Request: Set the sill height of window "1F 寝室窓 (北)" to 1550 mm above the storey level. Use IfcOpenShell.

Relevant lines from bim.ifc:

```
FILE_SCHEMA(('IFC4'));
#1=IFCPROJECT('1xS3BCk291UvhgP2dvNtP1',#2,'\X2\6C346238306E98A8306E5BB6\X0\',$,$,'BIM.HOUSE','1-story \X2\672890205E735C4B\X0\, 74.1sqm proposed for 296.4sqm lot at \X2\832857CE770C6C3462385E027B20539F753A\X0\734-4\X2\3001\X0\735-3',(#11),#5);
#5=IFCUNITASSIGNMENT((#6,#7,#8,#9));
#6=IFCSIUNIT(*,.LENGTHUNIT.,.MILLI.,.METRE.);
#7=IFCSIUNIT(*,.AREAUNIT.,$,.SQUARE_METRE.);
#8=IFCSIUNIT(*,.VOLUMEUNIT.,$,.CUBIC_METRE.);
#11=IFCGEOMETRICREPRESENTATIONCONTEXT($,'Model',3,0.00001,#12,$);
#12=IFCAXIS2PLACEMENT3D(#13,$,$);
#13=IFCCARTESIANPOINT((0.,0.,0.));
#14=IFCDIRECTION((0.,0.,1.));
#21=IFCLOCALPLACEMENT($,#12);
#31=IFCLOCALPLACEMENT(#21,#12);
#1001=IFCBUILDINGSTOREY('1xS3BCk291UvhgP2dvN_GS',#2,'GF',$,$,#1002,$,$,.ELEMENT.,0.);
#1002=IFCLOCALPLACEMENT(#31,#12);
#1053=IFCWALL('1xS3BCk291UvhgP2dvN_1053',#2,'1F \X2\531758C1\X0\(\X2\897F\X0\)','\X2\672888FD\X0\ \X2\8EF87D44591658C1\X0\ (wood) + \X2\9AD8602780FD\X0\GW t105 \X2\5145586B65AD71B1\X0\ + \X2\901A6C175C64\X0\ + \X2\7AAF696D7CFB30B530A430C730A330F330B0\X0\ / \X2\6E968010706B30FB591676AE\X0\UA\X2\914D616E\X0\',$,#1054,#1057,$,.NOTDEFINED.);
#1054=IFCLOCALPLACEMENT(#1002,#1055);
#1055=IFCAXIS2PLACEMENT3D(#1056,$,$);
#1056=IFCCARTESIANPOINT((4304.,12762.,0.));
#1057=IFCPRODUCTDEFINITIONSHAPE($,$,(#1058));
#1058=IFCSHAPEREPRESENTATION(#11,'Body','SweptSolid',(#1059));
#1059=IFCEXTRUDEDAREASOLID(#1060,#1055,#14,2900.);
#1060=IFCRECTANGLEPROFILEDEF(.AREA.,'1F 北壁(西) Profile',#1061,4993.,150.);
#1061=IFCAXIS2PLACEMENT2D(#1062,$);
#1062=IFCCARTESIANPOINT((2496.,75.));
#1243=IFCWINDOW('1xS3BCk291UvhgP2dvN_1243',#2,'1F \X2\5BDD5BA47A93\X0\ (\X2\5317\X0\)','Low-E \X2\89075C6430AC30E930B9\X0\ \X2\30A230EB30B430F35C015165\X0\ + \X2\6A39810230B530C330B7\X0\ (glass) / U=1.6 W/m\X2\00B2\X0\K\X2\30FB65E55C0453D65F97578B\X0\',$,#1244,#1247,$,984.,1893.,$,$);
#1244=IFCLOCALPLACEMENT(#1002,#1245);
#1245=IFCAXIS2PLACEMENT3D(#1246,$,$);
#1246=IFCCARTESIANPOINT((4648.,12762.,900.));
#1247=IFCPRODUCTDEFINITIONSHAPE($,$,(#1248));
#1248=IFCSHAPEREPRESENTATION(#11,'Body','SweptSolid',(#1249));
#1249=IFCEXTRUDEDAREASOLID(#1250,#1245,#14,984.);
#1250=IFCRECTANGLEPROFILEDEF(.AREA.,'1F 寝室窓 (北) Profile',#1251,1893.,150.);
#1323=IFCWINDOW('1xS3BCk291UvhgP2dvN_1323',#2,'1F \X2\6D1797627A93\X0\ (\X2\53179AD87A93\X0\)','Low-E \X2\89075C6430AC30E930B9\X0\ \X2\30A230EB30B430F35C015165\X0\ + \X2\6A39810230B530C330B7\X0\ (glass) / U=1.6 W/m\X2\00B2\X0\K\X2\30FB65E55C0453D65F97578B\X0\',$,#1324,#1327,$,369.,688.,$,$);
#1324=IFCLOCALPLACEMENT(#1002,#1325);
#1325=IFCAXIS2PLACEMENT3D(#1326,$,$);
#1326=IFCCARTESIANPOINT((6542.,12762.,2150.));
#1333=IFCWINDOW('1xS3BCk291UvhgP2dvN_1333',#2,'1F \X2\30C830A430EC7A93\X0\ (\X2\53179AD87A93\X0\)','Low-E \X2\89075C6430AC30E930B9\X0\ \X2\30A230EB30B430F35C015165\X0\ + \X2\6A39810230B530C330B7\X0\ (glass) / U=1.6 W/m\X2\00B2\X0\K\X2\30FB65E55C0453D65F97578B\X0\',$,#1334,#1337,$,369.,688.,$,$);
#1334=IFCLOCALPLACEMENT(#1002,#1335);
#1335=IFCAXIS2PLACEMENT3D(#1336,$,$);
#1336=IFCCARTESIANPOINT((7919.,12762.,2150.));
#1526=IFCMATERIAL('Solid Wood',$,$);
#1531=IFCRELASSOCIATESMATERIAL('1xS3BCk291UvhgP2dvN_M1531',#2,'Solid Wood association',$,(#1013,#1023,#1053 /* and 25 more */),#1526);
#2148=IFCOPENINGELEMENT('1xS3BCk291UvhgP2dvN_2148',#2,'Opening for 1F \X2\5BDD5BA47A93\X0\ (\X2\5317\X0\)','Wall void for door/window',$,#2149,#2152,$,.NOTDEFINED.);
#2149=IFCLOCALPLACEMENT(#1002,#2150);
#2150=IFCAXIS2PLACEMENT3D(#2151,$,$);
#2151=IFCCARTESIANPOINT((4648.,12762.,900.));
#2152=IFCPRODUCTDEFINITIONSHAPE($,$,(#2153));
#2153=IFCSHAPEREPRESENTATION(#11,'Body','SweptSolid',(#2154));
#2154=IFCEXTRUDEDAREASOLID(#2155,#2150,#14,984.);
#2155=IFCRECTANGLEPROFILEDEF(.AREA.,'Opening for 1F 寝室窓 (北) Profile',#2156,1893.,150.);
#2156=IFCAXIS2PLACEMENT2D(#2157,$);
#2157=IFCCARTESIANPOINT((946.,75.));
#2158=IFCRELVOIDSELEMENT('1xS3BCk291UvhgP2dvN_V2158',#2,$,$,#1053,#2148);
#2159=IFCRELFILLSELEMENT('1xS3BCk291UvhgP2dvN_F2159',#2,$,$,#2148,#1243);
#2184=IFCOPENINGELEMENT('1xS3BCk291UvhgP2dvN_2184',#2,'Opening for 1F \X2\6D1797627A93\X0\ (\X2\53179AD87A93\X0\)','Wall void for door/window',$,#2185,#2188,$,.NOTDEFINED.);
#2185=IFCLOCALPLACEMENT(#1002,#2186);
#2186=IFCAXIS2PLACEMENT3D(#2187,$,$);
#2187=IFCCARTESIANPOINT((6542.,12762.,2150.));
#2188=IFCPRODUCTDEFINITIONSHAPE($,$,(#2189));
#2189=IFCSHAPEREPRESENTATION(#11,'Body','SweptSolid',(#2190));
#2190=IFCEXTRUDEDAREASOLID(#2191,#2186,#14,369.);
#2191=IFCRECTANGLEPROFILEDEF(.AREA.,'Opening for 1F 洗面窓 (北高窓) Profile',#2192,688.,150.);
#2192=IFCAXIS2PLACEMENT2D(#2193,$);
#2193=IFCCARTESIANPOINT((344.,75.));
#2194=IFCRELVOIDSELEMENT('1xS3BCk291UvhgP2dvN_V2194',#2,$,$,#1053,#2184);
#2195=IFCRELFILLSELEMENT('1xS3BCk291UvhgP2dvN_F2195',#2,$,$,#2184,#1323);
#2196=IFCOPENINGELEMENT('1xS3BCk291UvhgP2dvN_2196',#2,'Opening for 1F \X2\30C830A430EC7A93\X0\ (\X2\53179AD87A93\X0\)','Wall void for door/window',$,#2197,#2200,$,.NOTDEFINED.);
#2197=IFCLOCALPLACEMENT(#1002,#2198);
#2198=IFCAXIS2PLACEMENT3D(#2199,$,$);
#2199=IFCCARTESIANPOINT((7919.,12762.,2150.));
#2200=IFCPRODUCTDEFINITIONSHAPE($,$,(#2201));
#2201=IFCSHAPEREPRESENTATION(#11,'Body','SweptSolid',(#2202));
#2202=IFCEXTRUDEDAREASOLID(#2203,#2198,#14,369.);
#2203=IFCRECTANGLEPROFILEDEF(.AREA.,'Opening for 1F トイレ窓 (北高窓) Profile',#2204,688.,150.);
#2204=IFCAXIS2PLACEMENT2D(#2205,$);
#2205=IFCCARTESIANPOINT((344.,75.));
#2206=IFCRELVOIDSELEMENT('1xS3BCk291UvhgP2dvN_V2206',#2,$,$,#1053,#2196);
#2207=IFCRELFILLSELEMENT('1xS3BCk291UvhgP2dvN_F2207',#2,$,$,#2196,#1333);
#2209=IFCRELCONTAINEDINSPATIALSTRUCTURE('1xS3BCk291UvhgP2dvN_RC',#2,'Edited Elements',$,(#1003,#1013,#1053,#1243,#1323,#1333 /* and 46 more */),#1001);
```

```python
import numpy as np
import ifcopenshell
import ifcopenshell.api.geometry
import ifcopenshell.geom
import ifcopenshell.util.element
import ifcopenshell.util.placement
import ifcopenshell.util.shape
import ifcopenshell.util.unit

model = ifcopenshell.open("bim.ifc")
unit_scale = ifcopenshell.util.unit.calculate_unit_scale(model)

window = model.by_guid("1xS3BCk291UvhgP2dvN_1243")
opening = window.FillsVoids[0].RelatingOpeningElement
storey = ifcopenshell.util.element.get_container(window, ifc_class="IfcBuildingStorey")
level = ifcopenshell.util.placement.get_local_placement(storey.ObjectPlacement)[2, 3]

# The opening's origin need not be at the sill, so measure its lowest point.
shape = ifcopenshell.geom.create_shape(ifcopenshell.geom.settings(), opening)
bottom = ifcopenshell.util.shape.get_shape_bottom_elevation(shape, shape.geometry) / unit_scale
dz = level + 1550.0 - bottom

shift = np.array([0.0, 0.0, dz])
# The window is not placed relative to its opening, so move both.
for product in (opening, window):
    matrix = ifcopenshell.util.placement.get_local_placement(product.ObjectPlacement)
    matrix[:3, 3] += shift
    ifcopenshell.api.geometry.edit_object_placement(model, product=product, matrix=matrix, is_si=False)

print(f"moved by {dz * unit_scale:+.3f} m")

model.write("bim_edited.ifc")
```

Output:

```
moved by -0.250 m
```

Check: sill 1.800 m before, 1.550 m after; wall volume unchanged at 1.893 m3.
